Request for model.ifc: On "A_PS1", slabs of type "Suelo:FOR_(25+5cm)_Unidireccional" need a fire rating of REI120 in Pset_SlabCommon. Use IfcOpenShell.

First a look at what the model holds.

```python
import ifcopenshell
import ifcopenshell.util.element

model = ifcopenshell.open("model.ifc")
print(model.schema)
storey = next(s for s in model.by_type("IfcBuildingStorey") if s.Name == "A_PS1")
slabs = [e for e in ifcopenshell.util.element.get_decomposition(storey) if e.is_a("IfcSlab")]
seen = {}
for e in slabs:
    element_type = ifcopenshell.util.element.get_type(e)
    key = (element_type.Name if element_type != e and element_type else None, ifcopenshell.util.element.get_pset(e, "Pset_SlabCommon", "FireRating"))
    seen[key] = seen.get(key, 0) + 1
for (name, value), count in sorted(seen.items(), key=str):
    print(count, "x", name, "|", value)
```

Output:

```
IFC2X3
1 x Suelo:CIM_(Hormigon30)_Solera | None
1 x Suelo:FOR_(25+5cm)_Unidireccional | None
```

```python
import ifcopenshell
import ifcopenshell.api.pset
import ifcopenshell.util.element

model = ifcopenshell.open("model.ifc")

storey = next(s for s in model.by_type("IfcBuildingStorey") if s.Name == "A_PS1")
slabs = [e for e in ifcopenshell.util.element.get_decomposition(storey) if e.is_a("IfcSlab")]

count = 0
for e in slabs:
    element_type = ifcopenshell.util.element.get_type(e)
    if element_type in (None, e) or element_type.Name != "Suelo:FOR_(25+5cm)_Unidireccional":
        continue
    # add_pset returns the element's existing set when there is one.
    pset = ifcopenshell.api.pset.add_pset(model, product=e, name="Pset_SlabCommon")
    ifcopenshell.api.pset.edit_pset(model, pset=pset, properties={"FireRating": "REI120"})
    count += 1

print(count, "slabs updated")

model.write("model_v2.ifc")
```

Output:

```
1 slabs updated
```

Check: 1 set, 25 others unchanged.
